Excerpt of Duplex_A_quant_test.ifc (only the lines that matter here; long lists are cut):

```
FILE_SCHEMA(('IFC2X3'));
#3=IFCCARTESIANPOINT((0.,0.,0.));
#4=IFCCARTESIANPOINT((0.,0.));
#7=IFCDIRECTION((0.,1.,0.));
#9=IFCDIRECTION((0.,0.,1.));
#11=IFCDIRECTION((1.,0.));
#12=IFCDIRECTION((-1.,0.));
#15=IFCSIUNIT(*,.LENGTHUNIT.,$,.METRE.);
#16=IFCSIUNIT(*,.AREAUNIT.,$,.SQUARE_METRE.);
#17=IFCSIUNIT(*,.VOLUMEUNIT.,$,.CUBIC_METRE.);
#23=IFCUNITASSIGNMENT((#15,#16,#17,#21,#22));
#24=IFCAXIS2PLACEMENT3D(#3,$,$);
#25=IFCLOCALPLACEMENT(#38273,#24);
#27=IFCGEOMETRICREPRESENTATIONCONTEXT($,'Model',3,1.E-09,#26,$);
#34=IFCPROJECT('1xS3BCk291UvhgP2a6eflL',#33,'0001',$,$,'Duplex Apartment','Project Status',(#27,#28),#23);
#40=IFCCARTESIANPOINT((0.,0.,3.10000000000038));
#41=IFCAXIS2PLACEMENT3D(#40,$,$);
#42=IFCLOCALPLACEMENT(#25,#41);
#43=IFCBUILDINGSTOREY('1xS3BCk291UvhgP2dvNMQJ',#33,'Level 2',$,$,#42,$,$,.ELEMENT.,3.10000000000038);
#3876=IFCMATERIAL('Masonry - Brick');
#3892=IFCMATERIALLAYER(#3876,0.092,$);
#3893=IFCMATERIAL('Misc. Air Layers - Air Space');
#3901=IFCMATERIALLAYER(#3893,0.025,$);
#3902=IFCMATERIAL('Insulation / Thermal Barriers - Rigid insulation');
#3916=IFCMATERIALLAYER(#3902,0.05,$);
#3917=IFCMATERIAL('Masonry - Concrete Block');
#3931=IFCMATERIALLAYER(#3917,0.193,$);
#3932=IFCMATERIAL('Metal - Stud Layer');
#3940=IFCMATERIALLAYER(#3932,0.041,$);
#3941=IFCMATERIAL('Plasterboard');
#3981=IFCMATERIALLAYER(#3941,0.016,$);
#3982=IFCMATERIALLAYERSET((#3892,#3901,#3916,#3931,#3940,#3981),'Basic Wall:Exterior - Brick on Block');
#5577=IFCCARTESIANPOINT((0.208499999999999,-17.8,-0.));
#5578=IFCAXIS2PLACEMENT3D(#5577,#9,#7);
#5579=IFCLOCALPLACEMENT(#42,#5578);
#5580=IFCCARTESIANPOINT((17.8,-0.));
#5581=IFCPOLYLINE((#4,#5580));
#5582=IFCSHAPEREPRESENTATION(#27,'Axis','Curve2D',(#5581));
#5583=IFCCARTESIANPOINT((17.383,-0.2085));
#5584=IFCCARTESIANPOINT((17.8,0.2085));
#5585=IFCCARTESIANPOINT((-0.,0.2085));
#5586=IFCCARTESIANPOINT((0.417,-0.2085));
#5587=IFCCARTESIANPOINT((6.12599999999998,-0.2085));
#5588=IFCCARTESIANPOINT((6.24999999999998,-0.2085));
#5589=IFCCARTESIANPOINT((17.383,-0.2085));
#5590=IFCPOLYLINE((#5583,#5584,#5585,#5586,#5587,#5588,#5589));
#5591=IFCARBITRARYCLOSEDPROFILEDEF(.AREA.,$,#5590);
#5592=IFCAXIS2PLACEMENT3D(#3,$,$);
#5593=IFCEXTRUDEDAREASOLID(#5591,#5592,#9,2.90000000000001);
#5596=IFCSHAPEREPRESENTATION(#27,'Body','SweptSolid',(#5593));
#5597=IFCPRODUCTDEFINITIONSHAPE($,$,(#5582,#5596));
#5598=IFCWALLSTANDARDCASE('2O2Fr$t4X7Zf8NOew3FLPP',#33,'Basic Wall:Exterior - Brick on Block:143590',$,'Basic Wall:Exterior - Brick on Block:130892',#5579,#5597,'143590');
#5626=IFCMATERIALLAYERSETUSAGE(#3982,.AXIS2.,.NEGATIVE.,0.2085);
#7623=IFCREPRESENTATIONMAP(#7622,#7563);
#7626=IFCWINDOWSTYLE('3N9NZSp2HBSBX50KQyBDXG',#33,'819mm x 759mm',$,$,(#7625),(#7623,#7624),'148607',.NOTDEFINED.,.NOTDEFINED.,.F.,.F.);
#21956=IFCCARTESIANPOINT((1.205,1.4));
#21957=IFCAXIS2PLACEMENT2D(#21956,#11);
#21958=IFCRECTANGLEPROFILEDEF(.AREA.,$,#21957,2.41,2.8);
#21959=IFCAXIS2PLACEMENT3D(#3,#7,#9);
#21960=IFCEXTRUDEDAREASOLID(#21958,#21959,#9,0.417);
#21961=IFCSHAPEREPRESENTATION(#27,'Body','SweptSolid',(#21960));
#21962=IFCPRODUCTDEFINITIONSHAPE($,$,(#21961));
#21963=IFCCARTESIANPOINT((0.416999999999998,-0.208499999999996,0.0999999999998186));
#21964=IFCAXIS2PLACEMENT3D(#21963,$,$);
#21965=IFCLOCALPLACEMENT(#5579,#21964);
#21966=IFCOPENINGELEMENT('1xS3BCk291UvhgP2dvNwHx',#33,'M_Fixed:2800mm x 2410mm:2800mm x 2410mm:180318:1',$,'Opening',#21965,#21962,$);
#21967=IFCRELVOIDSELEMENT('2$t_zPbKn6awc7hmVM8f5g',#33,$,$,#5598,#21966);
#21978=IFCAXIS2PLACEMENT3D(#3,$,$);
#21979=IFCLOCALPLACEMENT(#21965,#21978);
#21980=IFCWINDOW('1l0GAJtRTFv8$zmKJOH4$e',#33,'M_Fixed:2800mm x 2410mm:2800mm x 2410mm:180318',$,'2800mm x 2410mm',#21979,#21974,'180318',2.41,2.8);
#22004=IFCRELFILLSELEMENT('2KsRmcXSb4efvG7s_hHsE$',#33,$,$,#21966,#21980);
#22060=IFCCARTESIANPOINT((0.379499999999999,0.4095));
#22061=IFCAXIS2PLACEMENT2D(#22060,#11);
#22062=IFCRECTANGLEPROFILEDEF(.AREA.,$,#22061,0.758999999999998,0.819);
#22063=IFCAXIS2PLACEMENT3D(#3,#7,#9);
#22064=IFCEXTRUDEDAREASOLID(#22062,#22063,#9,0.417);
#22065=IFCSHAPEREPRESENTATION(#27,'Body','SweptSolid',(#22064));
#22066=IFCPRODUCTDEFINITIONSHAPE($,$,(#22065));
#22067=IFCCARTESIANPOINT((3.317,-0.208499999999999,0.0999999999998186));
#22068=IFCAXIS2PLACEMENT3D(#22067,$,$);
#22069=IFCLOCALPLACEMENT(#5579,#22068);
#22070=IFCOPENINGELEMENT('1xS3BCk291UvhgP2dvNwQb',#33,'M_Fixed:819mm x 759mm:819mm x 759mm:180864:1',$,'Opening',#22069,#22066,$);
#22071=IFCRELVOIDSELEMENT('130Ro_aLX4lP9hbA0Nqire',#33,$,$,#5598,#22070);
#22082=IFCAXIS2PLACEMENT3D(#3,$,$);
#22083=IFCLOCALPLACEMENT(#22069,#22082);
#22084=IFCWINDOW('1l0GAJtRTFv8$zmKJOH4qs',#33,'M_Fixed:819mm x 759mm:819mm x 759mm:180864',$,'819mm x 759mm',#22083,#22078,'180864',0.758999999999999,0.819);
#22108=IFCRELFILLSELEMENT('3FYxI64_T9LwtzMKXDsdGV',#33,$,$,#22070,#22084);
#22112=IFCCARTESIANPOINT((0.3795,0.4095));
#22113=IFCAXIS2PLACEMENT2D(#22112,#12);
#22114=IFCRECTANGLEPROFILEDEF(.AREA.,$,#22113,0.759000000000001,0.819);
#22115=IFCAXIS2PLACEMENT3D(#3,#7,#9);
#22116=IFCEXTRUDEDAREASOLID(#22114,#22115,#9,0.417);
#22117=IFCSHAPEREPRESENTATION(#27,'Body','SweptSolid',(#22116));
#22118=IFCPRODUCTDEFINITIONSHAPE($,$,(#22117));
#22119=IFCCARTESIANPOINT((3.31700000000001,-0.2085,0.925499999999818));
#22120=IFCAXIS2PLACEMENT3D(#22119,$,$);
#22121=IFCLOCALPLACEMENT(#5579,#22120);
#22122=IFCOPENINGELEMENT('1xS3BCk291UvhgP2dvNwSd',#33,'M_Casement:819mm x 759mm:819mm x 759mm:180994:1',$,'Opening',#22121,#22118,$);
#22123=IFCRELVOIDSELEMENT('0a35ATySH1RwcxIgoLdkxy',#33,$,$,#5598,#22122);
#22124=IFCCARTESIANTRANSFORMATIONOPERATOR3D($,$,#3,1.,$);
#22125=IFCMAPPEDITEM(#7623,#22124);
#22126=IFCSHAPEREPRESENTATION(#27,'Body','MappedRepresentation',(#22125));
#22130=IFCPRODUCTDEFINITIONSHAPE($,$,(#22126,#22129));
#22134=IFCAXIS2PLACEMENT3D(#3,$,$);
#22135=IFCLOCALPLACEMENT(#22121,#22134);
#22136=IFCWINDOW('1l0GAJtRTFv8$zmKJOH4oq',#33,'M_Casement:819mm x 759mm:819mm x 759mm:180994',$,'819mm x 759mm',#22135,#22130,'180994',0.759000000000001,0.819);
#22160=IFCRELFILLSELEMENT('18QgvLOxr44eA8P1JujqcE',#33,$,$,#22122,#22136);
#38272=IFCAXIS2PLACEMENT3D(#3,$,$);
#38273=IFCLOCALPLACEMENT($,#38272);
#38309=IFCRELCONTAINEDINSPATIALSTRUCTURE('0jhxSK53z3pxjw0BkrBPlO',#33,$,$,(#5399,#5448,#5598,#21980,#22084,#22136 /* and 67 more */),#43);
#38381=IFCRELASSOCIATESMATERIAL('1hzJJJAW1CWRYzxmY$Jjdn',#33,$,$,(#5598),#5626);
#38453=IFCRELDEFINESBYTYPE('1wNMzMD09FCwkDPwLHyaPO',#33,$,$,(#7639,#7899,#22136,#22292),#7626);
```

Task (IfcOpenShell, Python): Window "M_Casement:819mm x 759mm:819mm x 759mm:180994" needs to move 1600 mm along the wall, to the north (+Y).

```python
import ifcopenshell
import ifcopenshell.api.geometry
import ifcopenshell.util.placement

model = ifcopenshell.open("Duplex_A_quant_test.ifc")

window = model.by_guid("1l0GAJtRTFv8$zmKJOH4oq")
opening = window.FillsVoids[0].RelatingOpeningElement
wall = opening.VoidsElements[0].RelatingBuildingElement

wall_matrix = ifcopenshell.util.placement.get_local_placement(wall.ObjectPlacement)
shift = wall_matrix[:3, 0] * 1.6
before = ifcopenshell.util.placement.get_local_placement(window.ObjectPlacement)[:3, 3].copy()

# The window is placed relative to its opening, so it follows when the opening moves.
matrix = ifcopenshell.util.placement.get_local_placement(opening.ObjectPlacement)
matrix[:3, 3] += shift
ifcopenshell.api.geometry.edit_object_placement(
    model, product=opening, matrix=matrix, is_si=False, should_transform_children=True
)

after = ifcopenshell.util.placement.get_local_placement(window.ObjectPlacement)[:3, 3]
print("window moved by", (after - before).round(3) + 0.0)

model.write("Duplex_A_quant_test-out.ifc")
```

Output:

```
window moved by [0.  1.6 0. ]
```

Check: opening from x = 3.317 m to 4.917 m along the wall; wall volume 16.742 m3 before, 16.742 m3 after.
